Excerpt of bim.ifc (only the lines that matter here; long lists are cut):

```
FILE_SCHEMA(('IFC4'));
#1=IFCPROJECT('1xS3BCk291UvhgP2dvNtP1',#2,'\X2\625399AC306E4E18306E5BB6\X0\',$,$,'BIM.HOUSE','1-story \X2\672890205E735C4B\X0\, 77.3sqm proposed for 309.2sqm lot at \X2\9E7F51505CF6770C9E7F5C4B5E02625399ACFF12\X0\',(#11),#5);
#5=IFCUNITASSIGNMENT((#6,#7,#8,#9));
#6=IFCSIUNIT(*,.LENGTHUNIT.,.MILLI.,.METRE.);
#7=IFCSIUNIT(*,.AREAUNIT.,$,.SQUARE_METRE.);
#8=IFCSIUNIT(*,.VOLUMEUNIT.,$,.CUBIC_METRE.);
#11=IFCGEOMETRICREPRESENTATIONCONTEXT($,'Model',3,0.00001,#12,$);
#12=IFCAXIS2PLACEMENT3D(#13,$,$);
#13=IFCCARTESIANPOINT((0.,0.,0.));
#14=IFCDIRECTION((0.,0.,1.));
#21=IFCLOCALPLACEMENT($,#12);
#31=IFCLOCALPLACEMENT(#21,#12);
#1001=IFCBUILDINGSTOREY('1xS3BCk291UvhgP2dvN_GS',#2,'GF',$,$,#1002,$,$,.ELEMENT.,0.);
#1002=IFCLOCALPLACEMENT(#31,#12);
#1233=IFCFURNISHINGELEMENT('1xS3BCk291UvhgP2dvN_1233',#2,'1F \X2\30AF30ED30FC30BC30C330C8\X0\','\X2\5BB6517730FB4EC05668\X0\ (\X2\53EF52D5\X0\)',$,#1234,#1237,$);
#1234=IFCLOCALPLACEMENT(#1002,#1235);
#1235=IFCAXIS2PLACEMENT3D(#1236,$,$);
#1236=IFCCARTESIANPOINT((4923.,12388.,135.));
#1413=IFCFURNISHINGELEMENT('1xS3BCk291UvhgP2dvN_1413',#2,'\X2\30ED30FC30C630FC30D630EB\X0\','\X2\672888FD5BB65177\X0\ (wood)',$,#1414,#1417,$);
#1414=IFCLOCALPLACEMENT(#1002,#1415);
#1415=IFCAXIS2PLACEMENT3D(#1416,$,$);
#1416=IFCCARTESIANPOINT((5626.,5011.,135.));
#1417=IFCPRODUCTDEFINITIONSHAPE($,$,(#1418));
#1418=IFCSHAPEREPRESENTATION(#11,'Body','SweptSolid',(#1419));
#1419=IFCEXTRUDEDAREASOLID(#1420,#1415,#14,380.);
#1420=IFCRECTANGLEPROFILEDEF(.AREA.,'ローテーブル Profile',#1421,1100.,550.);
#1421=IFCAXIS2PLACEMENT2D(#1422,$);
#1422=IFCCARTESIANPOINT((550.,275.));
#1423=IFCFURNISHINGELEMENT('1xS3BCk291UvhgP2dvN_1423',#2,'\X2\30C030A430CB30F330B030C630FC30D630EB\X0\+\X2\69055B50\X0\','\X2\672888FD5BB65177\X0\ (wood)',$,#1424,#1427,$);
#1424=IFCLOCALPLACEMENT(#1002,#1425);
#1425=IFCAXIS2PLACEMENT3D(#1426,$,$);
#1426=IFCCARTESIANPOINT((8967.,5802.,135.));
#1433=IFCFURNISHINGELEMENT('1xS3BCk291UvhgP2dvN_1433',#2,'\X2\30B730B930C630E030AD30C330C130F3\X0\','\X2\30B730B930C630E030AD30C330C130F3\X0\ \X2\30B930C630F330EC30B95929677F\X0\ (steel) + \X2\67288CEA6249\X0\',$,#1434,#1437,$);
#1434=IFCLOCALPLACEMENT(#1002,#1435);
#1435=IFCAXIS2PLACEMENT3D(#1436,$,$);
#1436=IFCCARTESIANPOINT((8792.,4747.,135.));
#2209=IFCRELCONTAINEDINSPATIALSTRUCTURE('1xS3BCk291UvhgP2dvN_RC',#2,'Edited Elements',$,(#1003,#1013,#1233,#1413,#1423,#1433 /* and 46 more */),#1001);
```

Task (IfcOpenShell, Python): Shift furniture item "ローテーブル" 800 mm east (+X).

```python
import ifcopenshell
import ifcopenshell.api.geometry
import ifcopenshell.util.placement
import ifcopenshell.util.unit

model = ifcopenshell.open("bim.ifc")
unit_scale = ifcopenshell.util.unit.calculate_unit_scale(model)

item = model.by_id(1413)
matrix = ifcopenshell.util.placement.get_local_placement(item.ObjectPlacement)
matrix[0, 3] += 0.8 / unit_scale
ifcopenshell.api.geometry.edit_object_placement(model, product=item, matrix=matrix, is_si=False)

print(ifcopenshell.util.placement.get_local_placement(item.ObjectPlacement).round(3) + 0.0)

model.write("bim_updated.ifc")
```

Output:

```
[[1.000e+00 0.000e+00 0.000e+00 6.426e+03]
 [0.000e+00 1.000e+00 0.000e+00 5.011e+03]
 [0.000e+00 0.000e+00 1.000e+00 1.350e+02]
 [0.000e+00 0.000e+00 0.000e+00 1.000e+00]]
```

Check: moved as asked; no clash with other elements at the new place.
